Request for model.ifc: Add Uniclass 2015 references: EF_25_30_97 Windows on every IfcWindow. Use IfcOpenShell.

First a look at what the model holds.

```python
import ifcopenshell

model = ifcopenshell.open("model.ifc")
print(model.schema)
print("classifications:", [c.Name for c in model.by_type("IfcClassification")])
for ifc_class in ("IfcDoor", "IfcRoof", "IfcStair", "IfcWall", "IfcWindow"):
    print(ifc_class, len(model.by_type(ifc_class)))
```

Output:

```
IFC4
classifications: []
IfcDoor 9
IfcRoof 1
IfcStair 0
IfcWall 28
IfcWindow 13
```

```python
import ifcopenshell
import ifcopenshell.api.classification

model = ifcopenshell.open("model.ifc")

system = ifcopenshell.api.classification.add_classification(model, classification="Uniclass 2015")

codes = {
    "IfcWindow": ("EF_25_30_97", "Windows"),
}
for ifc_class, (code, name) in codes.items():
    products = model.by_type(ifc_class)
    ifcopenshell.api.classification.add_reference(
        model, products=products, classification=system, identification=code, name=name
    )
    print(code, len(products))

model.write("model_updated.ifc")
```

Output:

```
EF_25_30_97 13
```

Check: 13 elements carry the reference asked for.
